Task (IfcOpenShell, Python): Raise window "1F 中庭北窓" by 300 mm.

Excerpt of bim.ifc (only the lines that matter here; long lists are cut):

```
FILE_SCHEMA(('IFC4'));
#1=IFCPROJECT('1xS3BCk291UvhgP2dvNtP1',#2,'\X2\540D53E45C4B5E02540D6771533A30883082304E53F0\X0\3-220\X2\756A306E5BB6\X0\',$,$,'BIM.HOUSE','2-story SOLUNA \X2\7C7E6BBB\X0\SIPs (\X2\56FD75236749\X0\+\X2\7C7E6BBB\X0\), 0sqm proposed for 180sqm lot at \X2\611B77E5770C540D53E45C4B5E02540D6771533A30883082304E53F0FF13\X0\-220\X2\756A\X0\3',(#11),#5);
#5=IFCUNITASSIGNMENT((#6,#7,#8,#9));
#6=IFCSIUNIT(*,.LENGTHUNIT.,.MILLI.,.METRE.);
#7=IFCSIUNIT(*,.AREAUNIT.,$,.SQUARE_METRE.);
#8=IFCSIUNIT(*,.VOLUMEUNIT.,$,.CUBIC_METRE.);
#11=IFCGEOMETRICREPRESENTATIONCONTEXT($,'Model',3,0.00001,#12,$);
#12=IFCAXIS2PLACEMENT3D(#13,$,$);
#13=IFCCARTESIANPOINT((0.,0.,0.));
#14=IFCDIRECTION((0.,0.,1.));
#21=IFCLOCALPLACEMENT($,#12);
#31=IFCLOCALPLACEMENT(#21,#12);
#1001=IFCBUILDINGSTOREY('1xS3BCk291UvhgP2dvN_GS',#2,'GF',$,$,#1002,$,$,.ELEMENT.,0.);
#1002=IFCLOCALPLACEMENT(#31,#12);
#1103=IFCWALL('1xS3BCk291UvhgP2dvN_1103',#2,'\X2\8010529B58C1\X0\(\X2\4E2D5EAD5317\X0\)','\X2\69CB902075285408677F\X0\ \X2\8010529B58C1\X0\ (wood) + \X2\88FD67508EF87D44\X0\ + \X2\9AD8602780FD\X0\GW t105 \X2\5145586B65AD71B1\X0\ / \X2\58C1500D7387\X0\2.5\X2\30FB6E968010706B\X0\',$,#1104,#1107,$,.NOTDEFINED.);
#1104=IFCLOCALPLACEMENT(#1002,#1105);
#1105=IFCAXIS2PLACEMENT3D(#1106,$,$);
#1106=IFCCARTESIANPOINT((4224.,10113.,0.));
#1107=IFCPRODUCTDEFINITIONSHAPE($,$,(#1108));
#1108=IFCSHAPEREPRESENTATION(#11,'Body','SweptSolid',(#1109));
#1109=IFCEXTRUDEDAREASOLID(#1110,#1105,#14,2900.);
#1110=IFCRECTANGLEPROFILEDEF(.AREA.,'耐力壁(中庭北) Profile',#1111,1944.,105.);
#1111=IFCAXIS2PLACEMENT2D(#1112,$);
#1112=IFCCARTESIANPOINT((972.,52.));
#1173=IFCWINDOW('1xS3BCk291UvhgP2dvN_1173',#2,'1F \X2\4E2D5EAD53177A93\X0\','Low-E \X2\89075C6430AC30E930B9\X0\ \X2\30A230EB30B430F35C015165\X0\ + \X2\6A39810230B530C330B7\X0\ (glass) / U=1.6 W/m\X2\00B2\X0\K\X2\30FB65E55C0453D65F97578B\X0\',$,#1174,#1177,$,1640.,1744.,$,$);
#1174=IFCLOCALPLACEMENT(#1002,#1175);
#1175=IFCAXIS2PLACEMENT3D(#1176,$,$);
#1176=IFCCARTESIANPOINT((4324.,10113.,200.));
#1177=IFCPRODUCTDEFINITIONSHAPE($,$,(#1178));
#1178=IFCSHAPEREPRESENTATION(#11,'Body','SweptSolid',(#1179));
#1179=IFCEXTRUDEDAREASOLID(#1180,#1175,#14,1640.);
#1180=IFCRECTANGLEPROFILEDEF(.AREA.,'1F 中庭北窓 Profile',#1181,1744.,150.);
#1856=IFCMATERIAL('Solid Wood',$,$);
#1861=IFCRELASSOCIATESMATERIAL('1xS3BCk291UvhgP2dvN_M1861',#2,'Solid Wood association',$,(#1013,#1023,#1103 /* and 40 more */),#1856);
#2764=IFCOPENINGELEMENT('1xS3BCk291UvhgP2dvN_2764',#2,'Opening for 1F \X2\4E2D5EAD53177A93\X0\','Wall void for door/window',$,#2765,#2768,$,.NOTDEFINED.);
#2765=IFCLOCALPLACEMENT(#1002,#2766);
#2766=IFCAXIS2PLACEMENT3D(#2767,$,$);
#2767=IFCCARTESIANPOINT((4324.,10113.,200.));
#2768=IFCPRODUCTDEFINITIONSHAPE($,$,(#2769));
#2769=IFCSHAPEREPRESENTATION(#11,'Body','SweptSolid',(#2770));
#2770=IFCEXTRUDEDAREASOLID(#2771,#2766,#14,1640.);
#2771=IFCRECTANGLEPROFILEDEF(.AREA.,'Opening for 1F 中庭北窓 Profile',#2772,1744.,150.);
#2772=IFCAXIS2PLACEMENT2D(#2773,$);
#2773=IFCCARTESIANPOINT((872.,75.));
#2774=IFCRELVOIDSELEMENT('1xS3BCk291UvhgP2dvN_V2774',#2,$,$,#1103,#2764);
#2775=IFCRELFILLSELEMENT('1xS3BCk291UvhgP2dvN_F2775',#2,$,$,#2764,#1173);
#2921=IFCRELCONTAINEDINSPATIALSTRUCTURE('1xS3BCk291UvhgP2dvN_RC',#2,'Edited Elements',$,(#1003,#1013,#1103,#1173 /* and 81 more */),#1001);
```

```python
import numpy as np
import ifcopenshell
import ifcopenshell.api.geometry
import ifcopenshell.util.placement
import ifcopenshell.util.unit

model = ifcopenshell.open("bim.ifc")
unit_scale = ifcopenshell.util.unit.calculate_unit_scale(model)

window = model.by_guid("1xS3BCk291UvhgP2dvN_1173")
opening = window.FillsVoids[0].RelatingOpeningElement
dz = 0.3 / unit_scale

shift = np.array([0.0, 0.0, dz])
# The window is not placed relative to its opening, so move both.
for product in (opening, window):
    matrix = ifcopenshell.util.placement.get_local_placement(product.ObjectPlacement)
    matrix[:3, 3] += shift
    ifcopenshell.api.geometry.edit_object_placement(model, product=product, matrix=matrix, is_si=False)

print(f"moved by {dz * unit_scale:+.3f} m")

model.write("bim_rev.ifc")
```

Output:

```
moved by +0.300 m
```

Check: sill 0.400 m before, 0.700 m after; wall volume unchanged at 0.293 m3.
